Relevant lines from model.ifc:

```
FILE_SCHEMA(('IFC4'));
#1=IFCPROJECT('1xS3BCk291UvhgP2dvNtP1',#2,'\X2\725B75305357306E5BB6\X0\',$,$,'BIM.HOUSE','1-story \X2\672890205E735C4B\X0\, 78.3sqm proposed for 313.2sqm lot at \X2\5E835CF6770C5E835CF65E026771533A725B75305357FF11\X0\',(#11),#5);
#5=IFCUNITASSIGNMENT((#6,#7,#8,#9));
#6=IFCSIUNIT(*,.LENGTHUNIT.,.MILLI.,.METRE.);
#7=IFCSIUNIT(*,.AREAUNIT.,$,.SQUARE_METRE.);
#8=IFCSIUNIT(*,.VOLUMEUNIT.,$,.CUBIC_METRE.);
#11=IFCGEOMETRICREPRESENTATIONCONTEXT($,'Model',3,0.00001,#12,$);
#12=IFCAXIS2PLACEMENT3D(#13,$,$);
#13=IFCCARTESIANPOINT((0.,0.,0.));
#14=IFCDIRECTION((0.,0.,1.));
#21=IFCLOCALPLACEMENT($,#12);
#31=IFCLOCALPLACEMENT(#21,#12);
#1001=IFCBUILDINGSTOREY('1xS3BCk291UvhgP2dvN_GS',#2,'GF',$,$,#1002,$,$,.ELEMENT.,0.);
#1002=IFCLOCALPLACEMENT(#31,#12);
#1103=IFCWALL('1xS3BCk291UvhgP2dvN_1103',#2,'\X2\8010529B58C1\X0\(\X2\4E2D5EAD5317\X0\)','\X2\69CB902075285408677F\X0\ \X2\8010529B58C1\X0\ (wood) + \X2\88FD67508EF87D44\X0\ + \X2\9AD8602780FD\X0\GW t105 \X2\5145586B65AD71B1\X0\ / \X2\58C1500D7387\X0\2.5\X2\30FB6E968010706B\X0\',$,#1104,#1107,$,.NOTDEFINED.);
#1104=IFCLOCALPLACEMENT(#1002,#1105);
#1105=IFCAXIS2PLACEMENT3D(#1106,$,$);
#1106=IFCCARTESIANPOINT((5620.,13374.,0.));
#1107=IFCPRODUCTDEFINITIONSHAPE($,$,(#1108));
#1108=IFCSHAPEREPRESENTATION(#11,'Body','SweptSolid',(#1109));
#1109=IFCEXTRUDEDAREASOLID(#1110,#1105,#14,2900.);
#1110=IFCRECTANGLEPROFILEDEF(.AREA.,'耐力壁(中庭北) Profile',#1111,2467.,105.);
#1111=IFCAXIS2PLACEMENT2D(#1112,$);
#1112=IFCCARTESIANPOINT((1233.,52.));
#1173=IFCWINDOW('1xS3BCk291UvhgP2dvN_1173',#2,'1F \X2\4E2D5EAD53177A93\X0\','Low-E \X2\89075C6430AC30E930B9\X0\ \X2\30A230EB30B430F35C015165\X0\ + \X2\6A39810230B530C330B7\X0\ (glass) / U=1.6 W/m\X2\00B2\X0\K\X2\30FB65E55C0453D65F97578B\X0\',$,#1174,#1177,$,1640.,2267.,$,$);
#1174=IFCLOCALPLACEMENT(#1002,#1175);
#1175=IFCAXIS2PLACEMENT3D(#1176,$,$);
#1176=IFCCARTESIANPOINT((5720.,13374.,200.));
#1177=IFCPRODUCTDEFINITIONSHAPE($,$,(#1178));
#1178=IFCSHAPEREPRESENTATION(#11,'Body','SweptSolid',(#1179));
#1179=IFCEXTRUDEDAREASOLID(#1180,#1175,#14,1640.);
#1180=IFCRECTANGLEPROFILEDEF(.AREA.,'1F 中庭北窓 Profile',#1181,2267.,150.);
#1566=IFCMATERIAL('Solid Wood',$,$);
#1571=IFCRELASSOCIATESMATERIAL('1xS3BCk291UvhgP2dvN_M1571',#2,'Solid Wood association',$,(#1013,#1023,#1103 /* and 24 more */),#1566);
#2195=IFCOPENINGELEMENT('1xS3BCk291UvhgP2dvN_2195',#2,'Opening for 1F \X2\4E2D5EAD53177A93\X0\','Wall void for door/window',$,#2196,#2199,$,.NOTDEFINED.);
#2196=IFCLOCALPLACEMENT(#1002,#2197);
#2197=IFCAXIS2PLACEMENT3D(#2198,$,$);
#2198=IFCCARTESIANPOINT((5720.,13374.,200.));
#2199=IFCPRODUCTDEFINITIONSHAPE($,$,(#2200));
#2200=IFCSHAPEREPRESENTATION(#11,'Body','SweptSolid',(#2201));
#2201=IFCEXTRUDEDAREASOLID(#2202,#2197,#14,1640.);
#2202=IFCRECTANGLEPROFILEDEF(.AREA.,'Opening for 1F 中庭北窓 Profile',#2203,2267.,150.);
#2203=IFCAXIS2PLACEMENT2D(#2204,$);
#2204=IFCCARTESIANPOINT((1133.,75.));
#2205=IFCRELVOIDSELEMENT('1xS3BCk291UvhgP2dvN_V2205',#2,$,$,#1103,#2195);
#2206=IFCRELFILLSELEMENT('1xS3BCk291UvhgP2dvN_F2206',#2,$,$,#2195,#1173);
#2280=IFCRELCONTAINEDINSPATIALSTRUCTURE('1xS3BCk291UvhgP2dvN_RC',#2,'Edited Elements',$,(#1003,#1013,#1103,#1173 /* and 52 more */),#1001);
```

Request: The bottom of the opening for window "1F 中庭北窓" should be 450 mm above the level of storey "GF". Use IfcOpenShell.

```python
import numpy as np
import ifcopenshell
import ifcopenshell.api.geometry
import ifcopenshell.geom
import ifcopenshell.util.element
import ifcopenshell.util.placement
import ifcopenshell.util.shape
import ifcopenshell.util.unit

model = ifcopenshell.open("model.ifc")
unit_scale = ifcopenshell.util.unit.calculate_unit_scale(model)

window = model.by_guid("1xS3BCk291UvhgP2dvN_1173")
opening = window.FillsVoids[0].RelatingOpeningElement
storey = ifcopenshell.util.element.get_container(window, ifc_class="IfcBuildingStorey")
level = ifcopenshell.util.placement.get_local_placement(storey.ObjectPlacement)[2, 3]

# The opening's origin need not be at the sill, so measure its lowest point.
shape = ifcopenshell.geom.create_shape(ifcopenshell.geom.settings(), opening)
bottom = ifcopenshell.util.shape.get_shape_bottom_elevation(shape, shape.geometry) / unit_scale
dz = level + 450.0 - bottom

shift = np.array([0.0, 0.0, dz])
# The window is not placed relative to its opening, so move both.
for product in (opening, window):
    matrix = ifcopenshell.util.placement.get_local_placement(product.ObjectPlacement)
    matrix[:3, 3] += shift
    ifcopenshell.api.geometry.edit_object_placement(model, product=product, matrix=matrix, is_si=False)

print(f"moved by {dz * unit_scale:+.3f} m")

model.write("model_edited.ifc")
```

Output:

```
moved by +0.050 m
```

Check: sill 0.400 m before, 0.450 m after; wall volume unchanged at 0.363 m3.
